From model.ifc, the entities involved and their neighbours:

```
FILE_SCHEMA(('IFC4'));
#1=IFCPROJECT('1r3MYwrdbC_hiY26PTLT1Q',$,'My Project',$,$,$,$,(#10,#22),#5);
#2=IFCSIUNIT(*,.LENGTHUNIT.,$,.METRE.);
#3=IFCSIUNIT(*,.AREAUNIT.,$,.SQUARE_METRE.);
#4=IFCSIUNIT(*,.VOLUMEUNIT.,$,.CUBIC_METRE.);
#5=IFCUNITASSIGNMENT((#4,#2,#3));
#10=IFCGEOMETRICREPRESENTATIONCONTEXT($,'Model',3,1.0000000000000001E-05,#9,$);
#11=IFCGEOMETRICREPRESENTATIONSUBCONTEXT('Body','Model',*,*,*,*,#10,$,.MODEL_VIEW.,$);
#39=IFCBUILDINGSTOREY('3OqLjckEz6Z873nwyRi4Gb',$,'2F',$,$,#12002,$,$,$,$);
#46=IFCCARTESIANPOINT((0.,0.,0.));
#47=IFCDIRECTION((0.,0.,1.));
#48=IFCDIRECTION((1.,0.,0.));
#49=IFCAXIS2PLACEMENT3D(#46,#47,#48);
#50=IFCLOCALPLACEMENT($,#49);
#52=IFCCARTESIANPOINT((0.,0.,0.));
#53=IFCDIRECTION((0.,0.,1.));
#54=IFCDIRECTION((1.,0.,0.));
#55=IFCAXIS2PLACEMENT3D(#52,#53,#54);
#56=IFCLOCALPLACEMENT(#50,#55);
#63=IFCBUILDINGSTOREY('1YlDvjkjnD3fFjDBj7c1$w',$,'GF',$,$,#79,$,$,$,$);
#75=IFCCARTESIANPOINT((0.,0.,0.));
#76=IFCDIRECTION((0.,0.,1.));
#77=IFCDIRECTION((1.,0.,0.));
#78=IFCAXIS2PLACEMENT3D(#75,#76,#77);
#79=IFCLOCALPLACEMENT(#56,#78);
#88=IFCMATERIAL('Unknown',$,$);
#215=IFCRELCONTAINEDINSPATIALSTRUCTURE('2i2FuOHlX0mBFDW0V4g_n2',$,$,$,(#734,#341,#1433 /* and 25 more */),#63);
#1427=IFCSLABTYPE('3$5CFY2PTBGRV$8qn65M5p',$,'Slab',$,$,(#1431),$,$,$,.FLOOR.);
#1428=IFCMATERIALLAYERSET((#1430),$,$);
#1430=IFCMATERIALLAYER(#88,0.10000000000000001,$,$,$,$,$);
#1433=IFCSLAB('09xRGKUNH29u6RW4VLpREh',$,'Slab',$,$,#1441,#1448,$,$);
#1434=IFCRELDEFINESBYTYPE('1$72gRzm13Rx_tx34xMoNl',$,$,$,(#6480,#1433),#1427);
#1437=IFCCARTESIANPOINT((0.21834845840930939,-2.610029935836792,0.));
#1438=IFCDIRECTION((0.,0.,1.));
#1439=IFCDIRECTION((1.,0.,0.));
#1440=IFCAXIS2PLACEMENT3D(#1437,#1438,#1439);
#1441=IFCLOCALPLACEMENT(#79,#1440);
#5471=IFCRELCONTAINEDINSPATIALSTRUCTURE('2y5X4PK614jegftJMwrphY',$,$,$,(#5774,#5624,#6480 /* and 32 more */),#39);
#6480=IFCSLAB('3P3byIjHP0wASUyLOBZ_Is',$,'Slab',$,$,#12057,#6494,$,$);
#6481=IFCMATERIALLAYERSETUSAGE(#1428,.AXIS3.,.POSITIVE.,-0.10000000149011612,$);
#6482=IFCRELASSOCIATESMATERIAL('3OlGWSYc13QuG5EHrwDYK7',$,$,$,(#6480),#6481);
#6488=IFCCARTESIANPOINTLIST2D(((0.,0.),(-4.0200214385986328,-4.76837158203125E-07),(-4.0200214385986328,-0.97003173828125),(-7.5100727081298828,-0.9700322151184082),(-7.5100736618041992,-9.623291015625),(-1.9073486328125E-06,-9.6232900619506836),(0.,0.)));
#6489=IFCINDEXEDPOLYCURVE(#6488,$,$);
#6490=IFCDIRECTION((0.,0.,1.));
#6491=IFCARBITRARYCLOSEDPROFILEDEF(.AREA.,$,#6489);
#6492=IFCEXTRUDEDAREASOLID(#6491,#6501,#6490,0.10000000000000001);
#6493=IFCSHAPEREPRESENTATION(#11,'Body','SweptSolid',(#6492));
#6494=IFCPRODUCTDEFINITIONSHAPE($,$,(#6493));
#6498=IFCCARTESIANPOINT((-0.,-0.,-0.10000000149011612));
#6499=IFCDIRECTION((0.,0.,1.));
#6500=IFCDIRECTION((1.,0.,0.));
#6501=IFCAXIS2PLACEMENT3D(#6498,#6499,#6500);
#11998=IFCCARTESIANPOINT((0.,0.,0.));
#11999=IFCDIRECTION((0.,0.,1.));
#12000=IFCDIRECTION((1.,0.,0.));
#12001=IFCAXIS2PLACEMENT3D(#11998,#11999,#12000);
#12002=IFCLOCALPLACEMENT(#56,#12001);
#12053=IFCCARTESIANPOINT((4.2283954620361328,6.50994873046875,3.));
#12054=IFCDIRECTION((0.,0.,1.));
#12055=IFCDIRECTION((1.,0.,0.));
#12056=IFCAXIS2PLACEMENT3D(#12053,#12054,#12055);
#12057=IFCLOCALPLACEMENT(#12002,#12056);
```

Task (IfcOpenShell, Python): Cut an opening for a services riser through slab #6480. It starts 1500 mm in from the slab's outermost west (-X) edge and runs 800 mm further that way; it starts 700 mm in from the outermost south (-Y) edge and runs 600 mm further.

```python
import numpy as np
import ifcopenshell
import ifcopenshell.api.feature
import ifcopenshell.api.geometry
import ifcopenshell.api.root
import ifcopenshell.geom
import ifcopenshell.util.placement
import ifcopenshell.util.representation
import ifcopenshell.util.shape
import ifcopenshell.util.unit

model = ifcopenshell.open("model.ifc")
unit_scale = ifcopenshell.util.unit.calculate_unit_scale(model)
settings = ifcopenshell.geom.settings()


def volume(element):
    """Net volume in cubic metres, openings subtracted."""
    shape = ifcopenshell.geom.create_shape(settings, element)
    return ifcopenshell.util.shape.get_volume(shape.geometry)


slab = model.by_guid("3P3byIjHP0wASUyLOBZ_Is")
before = volume(slab)

# Extent in the slab's own axes, in metres. The edges named are its -X and -Y sides.
slab_shape = ifcopenshell.geom.create_shape(settings, slab)
vertices = ifcopenshell.util.shape.get_vertices(slab_shape.geometry)
x_min, y_min, bottom = vertices.min(axis=0)
top = vertices[:, 2].max()

opening = ifcopenshell.api.root.create_entity(model, ifc_class="IfcOpeningElement", name="Services riser opening", predefined_type="OPENING")
context = ifcopenshell.util.representation.get_context(model, "Model", "Body", "MODEL_VIEW")
width, depth = 0.8, 0.6
outline = [(0.0, 0.0), (width, 0.0), (width, depth), (0.0, depth), (0.0, 0.0)]
# Overshoot both faces by 50 mm so the cut is clean.
shape = ifcopenshell.api.geometry.add_slab_representation(
    model, context=context, depth=top - bottom + 0.1, polyline=outline
)
ifcopenshell.api.geometry.assign_representation(model, product=opening, representation=shape)

matrix = ifcopenshell.util.placement.get_local_placement(slab.ObjectPlacement)
matrix[:, 3] = matrix @ np.append(np.array([x_min + 1.5, y_min + 0.7, bottom - 0.05]) / unit_scale, 1.0)
ifcopenshell.api.geometry.edit_object_placement(model, product=opening, matrix=matrix, is_si=False)
ifcopenshell.api.feature.add_feature(model, feature=opening, element=slab)

after = volume(slab)

print(f"slab volume {before:.3f} -> {after:.3f} m3")

model.write("model_updated.ifc")
```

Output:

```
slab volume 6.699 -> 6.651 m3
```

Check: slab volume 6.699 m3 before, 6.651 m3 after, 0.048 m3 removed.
